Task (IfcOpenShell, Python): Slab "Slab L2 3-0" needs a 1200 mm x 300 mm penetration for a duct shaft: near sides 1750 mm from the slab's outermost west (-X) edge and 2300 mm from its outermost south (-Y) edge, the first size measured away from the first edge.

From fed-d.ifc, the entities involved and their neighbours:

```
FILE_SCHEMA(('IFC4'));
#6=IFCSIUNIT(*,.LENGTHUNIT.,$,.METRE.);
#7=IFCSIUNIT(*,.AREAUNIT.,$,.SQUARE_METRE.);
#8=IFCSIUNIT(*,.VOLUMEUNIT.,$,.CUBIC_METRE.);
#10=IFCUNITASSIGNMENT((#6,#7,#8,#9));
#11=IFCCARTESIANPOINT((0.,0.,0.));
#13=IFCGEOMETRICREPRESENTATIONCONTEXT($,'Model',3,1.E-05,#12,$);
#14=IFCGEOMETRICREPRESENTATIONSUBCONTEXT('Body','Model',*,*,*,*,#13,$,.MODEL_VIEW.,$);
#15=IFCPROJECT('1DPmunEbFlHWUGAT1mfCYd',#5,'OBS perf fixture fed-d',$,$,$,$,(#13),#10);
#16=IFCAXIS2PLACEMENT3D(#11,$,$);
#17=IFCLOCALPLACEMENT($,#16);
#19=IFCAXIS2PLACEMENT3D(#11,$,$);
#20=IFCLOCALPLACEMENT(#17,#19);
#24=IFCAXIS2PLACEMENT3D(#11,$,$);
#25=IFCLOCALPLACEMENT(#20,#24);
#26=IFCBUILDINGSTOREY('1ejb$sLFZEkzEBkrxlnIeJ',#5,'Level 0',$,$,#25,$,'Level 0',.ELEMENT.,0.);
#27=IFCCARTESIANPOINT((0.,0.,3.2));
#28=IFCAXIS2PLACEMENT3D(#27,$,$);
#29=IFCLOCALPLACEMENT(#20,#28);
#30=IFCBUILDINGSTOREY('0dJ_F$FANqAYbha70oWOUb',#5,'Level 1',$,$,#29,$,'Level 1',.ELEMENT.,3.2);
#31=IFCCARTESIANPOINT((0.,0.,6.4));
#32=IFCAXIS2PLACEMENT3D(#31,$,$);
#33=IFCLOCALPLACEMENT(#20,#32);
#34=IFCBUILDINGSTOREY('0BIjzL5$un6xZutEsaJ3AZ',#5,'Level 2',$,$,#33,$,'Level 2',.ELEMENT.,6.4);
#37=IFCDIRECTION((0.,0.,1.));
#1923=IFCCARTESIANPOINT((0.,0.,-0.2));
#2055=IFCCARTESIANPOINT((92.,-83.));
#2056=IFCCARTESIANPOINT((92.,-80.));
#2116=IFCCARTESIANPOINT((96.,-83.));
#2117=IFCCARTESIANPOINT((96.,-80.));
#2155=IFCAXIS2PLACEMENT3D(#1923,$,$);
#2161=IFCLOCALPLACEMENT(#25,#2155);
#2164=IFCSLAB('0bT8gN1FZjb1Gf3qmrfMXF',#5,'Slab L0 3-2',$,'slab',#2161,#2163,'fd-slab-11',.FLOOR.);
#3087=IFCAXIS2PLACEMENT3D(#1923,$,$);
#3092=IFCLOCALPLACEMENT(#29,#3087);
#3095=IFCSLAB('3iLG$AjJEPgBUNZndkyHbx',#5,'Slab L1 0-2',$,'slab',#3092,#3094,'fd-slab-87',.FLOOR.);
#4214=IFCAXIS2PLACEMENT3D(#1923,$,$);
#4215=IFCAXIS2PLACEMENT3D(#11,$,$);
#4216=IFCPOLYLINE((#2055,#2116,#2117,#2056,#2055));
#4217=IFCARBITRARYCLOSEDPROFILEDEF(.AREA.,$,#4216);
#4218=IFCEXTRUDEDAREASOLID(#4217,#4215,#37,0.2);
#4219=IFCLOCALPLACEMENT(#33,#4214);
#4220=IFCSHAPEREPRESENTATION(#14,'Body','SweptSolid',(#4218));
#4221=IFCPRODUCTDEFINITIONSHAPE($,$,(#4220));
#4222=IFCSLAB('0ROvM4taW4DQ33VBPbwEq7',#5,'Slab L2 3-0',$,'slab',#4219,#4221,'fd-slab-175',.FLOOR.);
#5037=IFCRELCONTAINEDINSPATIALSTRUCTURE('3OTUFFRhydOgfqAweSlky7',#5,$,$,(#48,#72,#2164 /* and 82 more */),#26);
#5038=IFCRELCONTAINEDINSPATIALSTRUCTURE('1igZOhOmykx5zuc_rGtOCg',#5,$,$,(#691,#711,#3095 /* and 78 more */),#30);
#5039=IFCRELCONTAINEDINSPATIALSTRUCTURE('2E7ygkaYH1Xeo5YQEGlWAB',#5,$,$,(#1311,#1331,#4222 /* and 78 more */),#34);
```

```python
import numpy as np
import ifcopenshell
import ifcopenshell.api.feature
import ifcopenshell.api.geometry
import ifcopenshell.api.root
import ifcopenshell.geom
import ifcopenshell.util.placement
import ifcopenshell.util.representation
import ifcopenshell.util.shape
import ifcopenshell.util.unit

model = ifcopenshell.open("fed-d.ifc")
unit_scale = ifcopenshell.util.unit.calculate_unit_scale(model)
settings = ifcopenshell.geom.settings()


def volume(element):
    """Net volume in cubic metres, openings subtracted."""
    shape = ifcopenshell.geom.create_shape(settings, element)
    return ifcopenshell.util.shape.get_volume(shape.geometry)


slab = model.by_id(4222)
before = volume(slab)

# Extent in the slab's own axes, in metres. The edges named are its -X and -Y sides.
slab_shape = ifcopenshell.geom.create_shape(settings, slab)
vertices = ifcopenshell.util.shape.get_vertices(slab_shape.geometry)
x_min, y_min, bottom = vertices.min(axis=0)
top = vertices[:, 2].max()

opening = ifcopenshell.api.root.create_entity(model, ifc_class="IfcOpeningElement", name="Duct shaft opening", predefined_type="OPENING")
context = ifcopenshell.util.representation.get_context(model, "Model", "Body", "MODEL_VIEW")
width, depth = 1.2, 0.3
outline = [(0.0, 0.0), (width, 0.0), (width, depth), (0.0, depth), (0.0, 0.0)]
# Overshoot both faces by 50 mm so the cut is clean.
shape = ifcopenshell.api.geometry.add_slab_representation(
    model, context=context, depth=top - bottom + 0.1, polyline=outline
)
ifcopenshell.api.geometry.assign_representation(model, product=opening, representation=shape)

matrix = ifcopenshell.util.placement.get_local_placement(slab.ObjectPlacement)
matrix[:, 3] = matrix @ np.append(np.array([x_min + 1.75, y_min + 2.3, bottom - 0.05]) / unit_scale, 1.0)
ifcopenshell.api.geometry.edit_object_placement(model, product=opening, matrix=matrix, is_si=False)
ifcopenshell.api.feature.add_feature(model, feature=opening, element=slab)

after = volume(slab)

print(f"slab volume {before:.3f} -> {after:.3f} m3")

model.write("fed-d_rev.ifc")
```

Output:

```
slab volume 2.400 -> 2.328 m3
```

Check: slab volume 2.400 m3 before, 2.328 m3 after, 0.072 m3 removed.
